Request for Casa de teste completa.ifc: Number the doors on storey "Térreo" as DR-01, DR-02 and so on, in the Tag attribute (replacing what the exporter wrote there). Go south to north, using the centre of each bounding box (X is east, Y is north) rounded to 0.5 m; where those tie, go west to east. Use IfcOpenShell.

First a look at what the model holds.

```python
import ifcopenshell
import ifcopenshell.util.element
import ifcopenshell.util.placement

model = ifcopenshell.open("Casa de teste completa.ifc")
print(model.schema)
storey = next(s for s in model.by_type("IfcBuildingStorey") if s.Name == "Térreo")
doors = [e for e in ifcopenshell.util.element.get_decomposition(storey) if e.is_a("IfcDoor")]
for e in sorted(doors, key=lambda e: e.id()):
    origin = ifcopenshell.util.placement.get_local_placement(e.ObjectPlacement)[:3, 3]
    print(e.id(), e.Tag, e.Name, origin.round(2) + 0.0, sep=" | ")
```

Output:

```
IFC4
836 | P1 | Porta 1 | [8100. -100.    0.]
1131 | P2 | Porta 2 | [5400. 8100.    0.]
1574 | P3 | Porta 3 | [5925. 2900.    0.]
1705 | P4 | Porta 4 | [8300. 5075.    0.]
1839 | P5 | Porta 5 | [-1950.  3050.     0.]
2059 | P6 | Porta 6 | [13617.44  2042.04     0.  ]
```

```python
import ifcopenshell
import ifcopenshell.geom
import ifcopenshell.util.element
import ifcopenshell.util.shape

model = ifcopenshell.open("Casa de teste completa.ifc")
settings = ifcopenshell.geom.settings()
settings.set("use-world-coords", True)


def centre(element):
    shape = ifcopenshell.geom.create_shape(settings, element)
    return ifcopenshell.util.shape.get_bbox_centroid(shape.geometry)


storey = next(s for s in model.by_type("IfcBuildingStorey") if s.Name == "Térreo")
doors = [e for e in ifcopenshell.util.element.get_decomposition(storey) if e.is_a("IfcDoor")]

# Insertion points can sit at a corner or the storey origin, so sort by the geometry (in metres).
centres = {e: centre(e) for e in doors}
doors.sort(key=lambda e: (round(centres[e][1] / 0.5), centres[e][0]))

for i, e in enumerate(doors, start=1):
    number = f"DR-{i:02d}"
    e.Tag = number
    print(e.id(), number)

model.write("Casa de teste completa_edited.ifc")
```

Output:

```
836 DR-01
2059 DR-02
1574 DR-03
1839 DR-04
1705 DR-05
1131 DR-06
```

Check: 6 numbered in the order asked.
